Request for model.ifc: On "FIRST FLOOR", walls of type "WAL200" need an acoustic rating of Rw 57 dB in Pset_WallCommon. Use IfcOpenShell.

First a look at what the model holds.

```python
import ifcopenshell
import ifcopenshell.util.element

model = ifcopenshell.open("model.ifc")
print(model.schema)
storey = next(s for s in model.by_type("IfcBuildingStorey") if s.Name == "FIRST FLOOR")
walls = [e for e in ifcopenshell.util.element.get_decomposition(storey) if e.is_a("IfcWall")]
seen = {}
for e in walls:
    element_type = ifcopenshell.util.element.get_type(e)
    key = (element_type.Name if element_type != e and element_type else None, ifcopenshell.util.element.get_pset(e, "Pset_WallCommon", "AcousticRating"))
    seen[key] = seen.get(key, 0) + 1
for (name, value), count in sorted(seen.items(), key=str):
    print(count, "x", name, "|", value)
```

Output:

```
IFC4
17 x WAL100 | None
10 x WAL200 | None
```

```python
import ifcopenshell
import ifcopenshell.api.pset
import ifcopenshell.util.element

model = ifcopenshell.open("model.ifc")

storey = next(s for s in model.by_type("IfcBuildingStorey") if s.Name == "FIRST FLOOR")
walls = [e for e in ifcopenshell.util.element.get_decomposition(storey) if e.is_a("IfcWall")]

count = 0
for e in walls:
    element_type = ifcopenshell.util.element.get_type(e)
    if element_type in (None, e) or element_type.Name != "WAL200":
        continue
    # add_pset returns the element's existing set when there is one.
    pset = ifcopenshell.api.pset.add_pset(model, product=e, name="Pset_WallCommon")
    ifcopenshell.api.pset.edit_pset(model, pset=pset, properties={"AcousticRating": "Rw 57 dB"})
    count += 1

print(count, "walls updated")

model.write("model_updated.ifc")
```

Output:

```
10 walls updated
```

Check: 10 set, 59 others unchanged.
